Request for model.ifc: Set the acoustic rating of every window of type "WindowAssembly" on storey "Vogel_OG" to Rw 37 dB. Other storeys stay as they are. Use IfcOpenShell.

First a look at what the model holds.

```python
import ifcopenshell
import ifcopenshell.util.element

model = ifcopenshell.open("model.ifc")
print(model.schema)
storey = next(s for s in model.by_type("IfcBuildingStorey") if s.Name == "Vogel_OG")
windows = [e for e in ifcopenshell.util.element.get_decomposition(storey) if e.is_a("IfcWindow")]
seen = {}
for e in windows:
    element_type = ifcopenshell.util.element.get_type(e)
    key = (element_type.Name if element_type != e and element_type else None, ifcopenshell.util.element.get_pset(e, "Pset_WindowCommon", "AcousticRating"))
    seen[key] = seen.get(key, 0) + 1
for (name, value), count in sorted(seen.items(), key=str):
    print(count, "x", name, "|", value)
```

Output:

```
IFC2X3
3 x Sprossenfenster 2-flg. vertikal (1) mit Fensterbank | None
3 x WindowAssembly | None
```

```python
import ifcopenshell
import ifcopenshell.api.pset
import ifcopenshell.util.element

model = ifcopenshell.open("model.ifc")

storey = next(s for s in model.by_type("IfcBuildingStorey") if s.Name == "Vogel_OG")
windows = [e for e in ifcopenshell.util.element.get_decomposition(storey) if e.is_a("IfcWindow")]

count = 0
for e in windows:
    element_type = ifcopenshell.util.element.get_type(e)
    if element_type in (None, e) or element_type.Name != "WindowAssembly":
        continue
    # add_pset returns the element's existing set when there is one.
    pset = ifcopenshell.api.pset.add_pset(model, product=e, name="Pset_WindowCommon")
    ifcopenshell.api.pset.edit_pset(model, pset=pset, properties={"AcousticRating": "Rw 37 dB"})
    count += 1

print(count, "windows updated")

model.write("model_updated.ifc")
```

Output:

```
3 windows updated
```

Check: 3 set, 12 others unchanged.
